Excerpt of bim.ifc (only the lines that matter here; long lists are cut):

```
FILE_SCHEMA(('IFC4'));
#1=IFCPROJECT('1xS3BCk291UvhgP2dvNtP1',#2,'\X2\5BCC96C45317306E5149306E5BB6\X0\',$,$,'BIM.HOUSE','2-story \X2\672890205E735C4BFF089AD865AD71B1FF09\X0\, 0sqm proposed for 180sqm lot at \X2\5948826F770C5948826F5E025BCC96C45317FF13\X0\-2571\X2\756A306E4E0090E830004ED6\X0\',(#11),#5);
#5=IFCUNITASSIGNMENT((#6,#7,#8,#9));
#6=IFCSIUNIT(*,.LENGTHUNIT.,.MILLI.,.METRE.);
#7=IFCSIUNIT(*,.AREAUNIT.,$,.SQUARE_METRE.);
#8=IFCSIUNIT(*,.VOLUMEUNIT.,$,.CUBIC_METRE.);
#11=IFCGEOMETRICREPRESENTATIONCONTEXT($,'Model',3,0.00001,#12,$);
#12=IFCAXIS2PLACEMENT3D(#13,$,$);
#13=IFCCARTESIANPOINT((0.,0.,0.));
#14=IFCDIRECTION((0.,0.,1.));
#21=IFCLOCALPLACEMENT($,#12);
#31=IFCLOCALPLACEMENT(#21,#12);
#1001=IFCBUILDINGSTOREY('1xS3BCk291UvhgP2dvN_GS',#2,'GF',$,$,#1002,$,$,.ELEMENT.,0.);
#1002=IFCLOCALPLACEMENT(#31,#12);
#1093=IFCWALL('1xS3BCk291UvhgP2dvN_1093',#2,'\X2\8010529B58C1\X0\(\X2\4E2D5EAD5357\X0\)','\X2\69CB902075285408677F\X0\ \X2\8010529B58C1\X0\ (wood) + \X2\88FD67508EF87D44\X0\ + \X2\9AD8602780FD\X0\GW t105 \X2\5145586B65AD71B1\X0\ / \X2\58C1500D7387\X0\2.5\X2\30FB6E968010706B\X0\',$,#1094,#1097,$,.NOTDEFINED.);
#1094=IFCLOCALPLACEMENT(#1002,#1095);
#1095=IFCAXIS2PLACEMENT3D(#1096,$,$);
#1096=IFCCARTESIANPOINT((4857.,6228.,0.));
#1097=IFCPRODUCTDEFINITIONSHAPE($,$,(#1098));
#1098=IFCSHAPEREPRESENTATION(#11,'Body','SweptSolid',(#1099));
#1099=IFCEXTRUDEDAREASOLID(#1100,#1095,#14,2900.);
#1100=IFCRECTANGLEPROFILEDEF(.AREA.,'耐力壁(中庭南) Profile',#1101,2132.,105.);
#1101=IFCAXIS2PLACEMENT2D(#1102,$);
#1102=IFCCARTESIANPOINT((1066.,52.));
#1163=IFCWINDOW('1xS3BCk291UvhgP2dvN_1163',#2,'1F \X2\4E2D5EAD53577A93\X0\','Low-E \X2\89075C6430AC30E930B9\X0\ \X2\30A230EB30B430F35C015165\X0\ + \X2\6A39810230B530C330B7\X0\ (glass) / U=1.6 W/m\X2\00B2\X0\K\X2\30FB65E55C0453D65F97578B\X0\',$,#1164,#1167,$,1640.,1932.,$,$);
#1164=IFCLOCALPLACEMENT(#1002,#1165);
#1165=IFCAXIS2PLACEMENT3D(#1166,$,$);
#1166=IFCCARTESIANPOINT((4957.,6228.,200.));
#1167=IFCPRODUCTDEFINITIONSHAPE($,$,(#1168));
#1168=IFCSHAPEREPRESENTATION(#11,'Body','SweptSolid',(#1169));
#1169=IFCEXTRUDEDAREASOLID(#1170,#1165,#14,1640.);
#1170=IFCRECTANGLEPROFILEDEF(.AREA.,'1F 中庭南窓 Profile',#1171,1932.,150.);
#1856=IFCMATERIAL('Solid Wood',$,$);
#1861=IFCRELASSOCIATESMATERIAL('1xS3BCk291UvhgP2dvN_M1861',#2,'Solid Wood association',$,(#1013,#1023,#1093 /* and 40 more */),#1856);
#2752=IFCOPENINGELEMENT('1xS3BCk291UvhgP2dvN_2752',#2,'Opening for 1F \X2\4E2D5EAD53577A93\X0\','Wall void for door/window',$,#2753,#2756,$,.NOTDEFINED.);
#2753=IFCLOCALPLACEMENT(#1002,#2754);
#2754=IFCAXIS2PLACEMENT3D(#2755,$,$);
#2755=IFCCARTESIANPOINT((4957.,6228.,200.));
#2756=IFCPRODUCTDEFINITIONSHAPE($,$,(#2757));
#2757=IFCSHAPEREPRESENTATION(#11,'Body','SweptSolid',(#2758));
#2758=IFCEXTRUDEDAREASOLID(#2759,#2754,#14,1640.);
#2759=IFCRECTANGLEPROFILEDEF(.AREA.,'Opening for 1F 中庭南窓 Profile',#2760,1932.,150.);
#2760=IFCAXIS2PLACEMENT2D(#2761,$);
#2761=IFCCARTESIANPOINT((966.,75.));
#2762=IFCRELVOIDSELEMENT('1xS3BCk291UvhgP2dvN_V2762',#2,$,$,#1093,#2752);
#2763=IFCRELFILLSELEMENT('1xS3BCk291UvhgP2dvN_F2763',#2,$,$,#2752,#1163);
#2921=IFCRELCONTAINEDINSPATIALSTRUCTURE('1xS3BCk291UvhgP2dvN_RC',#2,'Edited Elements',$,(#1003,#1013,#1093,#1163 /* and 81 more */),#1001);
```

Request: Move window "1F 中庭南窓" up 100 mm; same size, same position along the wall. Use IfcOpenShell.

```python
import numpy as np
import ifcopenshell
import ifcopenshell.api.geometry
import ifcopenshell.util.placement
import ifcopenshell.util.unit

model = ifcopenshell.open("bim.ifc")
unit_scale = ifcopenshell.util.unit.calculate_unit_scale(model)

window = model.by_guid("1xS3BCk291UvhgP2dvN_1163")
opening = window.FillsVoids[0].RelatingOpeningElement
dz = 100.0

shift = np.array([0.0, 0.0, dz])
# The window is not placed relative to its opening, so move both.
for product in (opening, window):
    matrix = ifcopenshell.util.placement.get_local_placement(product.ObjectPlacement)
    matrix[:3, 3] += shift
    ifcopenshell.api.geometry.edit_object_placement(model, product=product, matrix=matrix, is_si=False)

print(f"moved by {dz * unit_scale:+.3f} m")

model.write("bim_v2.ifc")
```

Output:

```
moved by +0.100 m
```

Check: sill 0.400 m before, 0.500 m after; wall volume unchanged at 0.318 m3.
